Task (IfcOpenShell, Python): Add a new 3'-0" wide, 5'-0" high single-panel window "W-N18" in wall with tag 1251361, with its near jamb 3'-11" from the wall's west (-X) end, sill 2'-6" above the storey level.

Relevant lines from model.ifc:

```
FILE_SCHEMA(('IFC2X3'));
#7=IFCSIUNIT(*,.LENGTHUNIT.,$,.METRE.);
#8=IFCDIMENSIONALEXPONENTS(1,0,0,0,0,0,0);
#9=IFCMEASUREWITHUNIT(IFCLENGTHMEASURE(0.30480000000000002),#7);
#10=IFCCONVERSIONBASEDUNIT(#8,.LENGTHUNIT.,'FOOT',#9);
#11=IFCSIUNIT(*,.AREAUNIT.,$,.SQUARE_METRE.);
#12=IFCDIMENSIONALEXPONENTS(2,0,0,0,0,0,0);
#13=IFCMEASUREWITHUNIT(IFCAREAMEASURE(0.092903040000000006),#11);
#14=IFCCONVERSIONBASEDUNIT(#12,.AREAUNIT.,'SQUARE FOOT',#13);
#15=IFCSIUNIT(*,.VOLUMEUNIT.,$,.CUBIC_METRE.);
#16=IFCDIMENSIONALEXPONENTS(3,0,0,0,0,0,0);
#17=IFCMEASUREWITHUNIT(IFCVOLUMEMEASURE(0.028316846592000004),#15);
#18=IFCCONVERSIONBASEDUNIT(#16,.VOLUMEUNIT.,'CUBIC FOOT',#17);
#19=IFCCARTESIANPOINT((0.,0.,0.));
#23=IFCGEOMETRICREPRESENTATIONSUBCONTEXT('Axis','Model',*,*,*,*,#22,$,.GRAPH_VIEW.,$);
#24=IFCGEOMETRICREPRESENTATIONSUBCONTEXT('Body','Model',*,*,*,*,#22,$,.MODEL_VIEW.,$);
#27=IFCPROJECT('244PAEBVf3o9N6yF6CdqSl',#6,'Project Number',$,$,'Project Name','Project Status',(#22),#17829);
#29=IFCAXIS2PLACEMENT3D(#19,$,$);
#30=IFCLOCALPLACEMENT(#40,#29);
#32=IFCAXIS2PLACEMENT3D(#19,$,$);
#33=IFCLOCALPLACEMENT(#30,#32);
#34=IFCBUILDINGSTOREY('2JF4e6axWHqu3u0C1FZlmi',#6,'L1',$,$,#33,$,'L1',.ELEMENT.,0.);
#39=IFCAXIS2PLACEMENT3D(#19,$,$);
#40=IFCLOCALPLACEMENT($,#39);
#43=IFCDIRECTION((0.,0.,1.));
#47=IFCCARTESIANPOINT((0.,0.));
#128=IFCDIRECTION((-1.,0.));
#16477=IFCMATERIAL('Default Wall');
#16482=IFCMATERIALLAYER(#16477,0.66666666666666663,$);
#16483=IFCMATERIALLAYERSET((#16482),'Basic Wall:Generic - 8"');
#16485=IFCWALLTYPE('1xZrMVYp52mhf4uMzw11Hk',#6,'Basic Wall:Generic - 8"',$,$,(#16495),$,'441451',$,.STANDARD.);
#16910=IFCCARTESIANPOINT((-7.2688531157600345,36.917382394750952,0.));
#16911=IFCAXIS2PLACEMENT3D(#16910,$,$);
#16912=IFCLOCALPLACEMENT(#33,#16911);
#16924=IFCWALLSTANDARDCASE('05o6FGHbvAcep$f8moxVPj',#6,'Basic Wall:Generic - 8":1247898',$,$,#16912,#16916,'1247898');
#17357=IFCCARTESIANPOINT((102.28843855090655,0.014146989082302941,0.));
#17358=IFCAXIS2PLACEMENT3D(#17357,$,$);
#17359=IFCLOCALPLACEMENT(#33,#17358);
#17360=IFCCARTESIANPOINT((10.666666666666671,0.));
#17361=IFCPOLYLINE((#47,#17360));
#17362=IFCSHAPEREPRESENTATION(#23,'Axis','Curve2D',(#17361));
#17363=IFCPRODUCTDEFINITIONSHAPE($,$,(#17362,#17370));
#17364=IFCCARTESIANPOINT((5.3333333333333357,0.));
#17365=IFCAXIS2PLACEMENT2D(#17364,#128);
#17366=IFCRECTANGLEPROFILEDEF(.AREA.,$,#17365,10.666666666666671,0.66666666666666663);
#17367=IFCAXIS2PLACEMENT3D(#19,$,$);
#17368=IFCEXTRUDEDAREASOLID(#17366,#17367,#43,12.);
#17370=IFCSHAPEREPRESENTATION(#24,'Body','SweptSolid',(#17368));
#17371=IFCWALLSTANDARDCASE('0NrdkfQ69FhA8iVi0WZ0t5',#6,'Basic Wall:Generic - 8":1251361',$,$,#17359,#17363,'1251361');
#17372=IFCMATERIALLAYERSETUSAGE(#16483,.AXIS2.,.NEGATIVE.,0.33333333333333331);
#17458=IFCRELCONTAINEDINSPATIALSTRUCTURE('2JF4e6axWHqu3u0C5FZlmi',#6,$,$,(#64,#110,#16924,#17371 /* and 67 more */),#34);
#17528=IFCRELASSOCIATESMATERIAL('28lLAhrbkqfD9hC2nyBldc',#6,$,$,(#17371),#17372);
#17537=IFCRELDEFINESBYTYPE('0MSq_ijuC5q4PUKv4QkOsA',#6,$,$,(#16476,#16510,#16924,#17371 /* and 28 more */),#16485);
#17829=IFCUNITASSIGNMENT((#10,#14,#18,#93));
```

```python
import numpy as np
import ifcopenshell
import ifcopenshell.api.feature
import ifcopenshell.api.geometry
import ifcopenshell.api.root
import ifcopenshell.api.spatial
import ifcopenshell.api.type
import ifcopenshell.geom
import ifcopenshell.util.element
import ifcopenshell.util.placement
import ifcopenshell.util.representation
import ifcopenshell.util.shape
import ifcopenshell.util.unit

model = ifcopenshell.open("model.ifc")
unit_scale = ifcopenshell.util.unit.calculate_unit_scale(model)
settings = ifcopenshell.geom.settings()


def volume(element):
    """Net volume in cubic metres, openings subtracted."""
    shape = ifcopenshell.geom.create_shape(settings, element)
    return ifcopenshell.util.shape.get_volume(shape.geometry)


wall = model.by_guid("0NrdkfQ69FhA8iVi0WZ0t5")
storey = ifcopenshell.util.element.get_container(wall, ifc_class="IfcBuildingStorey")
context = ifcopenshell.util.representation.get_context(model, "Model", "Body", "MODEL_VIEW")
before = volume(wall)

width, height, from_end, sill = 0.9144, 1.524, 1.1938, 0.762  # metres

# The wall runs along its own X axis, and the end named is its -X end.
wall_shape = ifcopenshell.geom.create_shape(settings, wall)
x, y, z = ifcopenshell.util.shape.get_vertices(wall_shape.geometry).T
start = x.min() + from_end
face, thickness = float(y.min()), float(y.max() - y.min())
wall_matrix = ifcopenshell.util.placement.get_local_placement(wall.ObjectPlacement)
level = ifcopenshell.util.placement.get_local_placement(storey.ObjectPlacement)[2, 3]


def in_wall(x, y):
    """Placement at x, y metres in the wall's axes, at sill height."""
    matrix = wall_matrix.copy()
    matrix[:, 3] = wall_matrix @ np.array([x / unit_scale, y / unit_scale, 0.0, 1.0])
    matrix[2, 3] = level + sill / unit_scale
    return matrix


# Opening: a box that overshoots both wall faces by 50 mm.
opening = ifcopenshell.api.root.create_entity(model, ifc_class="IfcOpeningElement")
box = ifcopenshell.api.geometry.add_wall_representation(
    model, context=context, length=width, height=height, thickness=thickness + 0.1
)
ifcopenshell.api.geometry.assign_representation(model, product=opening, representation=box)
ifcopenshell.api.geometry.edit_object_placement(model, product=opening, matrix=in_wall(start, face - 0.05), is_si=False)
ifcopenshell.api.feature.add_feature(model, feature=opening, element=wall)

window = ifcopenshell.api.root.create_entity(model, ifc_class="IfcWindow", name="W-N18")
window.OverallWidth, window.OverallHeight = width / unit_scale, height / unit_scale
body = ifcopenshell.api.geometry.add_window_representation(
    model,
    context=context,
    overall_width=window.OverallWidth,
    overall_height=window.OverallHeight,
    partition_type="SINGLE_PANEL",
)
ifcopenshell.api.geometry.assign_representation(model, product=window, representation=body)
ifcopenshell.api.spatial.assign_container(model, products=[window], relating_structure=storey)
fills = ifcopenshell.api.feature.add_filling(model, opening=opening, element=window)
fills.OwnerHistory = window.OwnerHistory  # required in IFC2X3

# IFC2X3 keeps the operation on the window style.
style = ifcopenshell.api.root.create_entity(model, ifc_class="IfcWindowStyle", name="W-N18")
style.OperationType, style.ConstructionType = "SINGLE_PANEL", "NOTDEFINED"
style.ParameterTakesPrecedence = style.Sizeable = False
ifcopenshell.api.type.assign_type(model, related_objects=[window], relating_type=style)

# Centre the window in the wall's thickness.
ifcopenshell.api.geometry.edit_object_placement(model, product=window, matrix=in_wall(start, face), is_si=False)
window_shape = ifcopenshell.geom.create_shape(settings, window)
depth = ifcopenshell.util.shape.get_vertices(window_shape.geometry)[:, 1]
offset = face + thickness / 2 - (depth.min() + depth.max()) / 2
ifcopenshell.api.geometry.edit_object_placement(model, product=window, matrix=in_wall(start, offset), is_si=False)

after = volume(wall)

print(f"wall volume {before:.3f} -> {after:.3f} m3")

model.write("model_v2.ifc")
```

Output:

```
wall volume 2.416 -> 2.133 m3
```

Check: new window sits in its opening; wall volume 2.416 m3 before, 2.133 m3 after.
